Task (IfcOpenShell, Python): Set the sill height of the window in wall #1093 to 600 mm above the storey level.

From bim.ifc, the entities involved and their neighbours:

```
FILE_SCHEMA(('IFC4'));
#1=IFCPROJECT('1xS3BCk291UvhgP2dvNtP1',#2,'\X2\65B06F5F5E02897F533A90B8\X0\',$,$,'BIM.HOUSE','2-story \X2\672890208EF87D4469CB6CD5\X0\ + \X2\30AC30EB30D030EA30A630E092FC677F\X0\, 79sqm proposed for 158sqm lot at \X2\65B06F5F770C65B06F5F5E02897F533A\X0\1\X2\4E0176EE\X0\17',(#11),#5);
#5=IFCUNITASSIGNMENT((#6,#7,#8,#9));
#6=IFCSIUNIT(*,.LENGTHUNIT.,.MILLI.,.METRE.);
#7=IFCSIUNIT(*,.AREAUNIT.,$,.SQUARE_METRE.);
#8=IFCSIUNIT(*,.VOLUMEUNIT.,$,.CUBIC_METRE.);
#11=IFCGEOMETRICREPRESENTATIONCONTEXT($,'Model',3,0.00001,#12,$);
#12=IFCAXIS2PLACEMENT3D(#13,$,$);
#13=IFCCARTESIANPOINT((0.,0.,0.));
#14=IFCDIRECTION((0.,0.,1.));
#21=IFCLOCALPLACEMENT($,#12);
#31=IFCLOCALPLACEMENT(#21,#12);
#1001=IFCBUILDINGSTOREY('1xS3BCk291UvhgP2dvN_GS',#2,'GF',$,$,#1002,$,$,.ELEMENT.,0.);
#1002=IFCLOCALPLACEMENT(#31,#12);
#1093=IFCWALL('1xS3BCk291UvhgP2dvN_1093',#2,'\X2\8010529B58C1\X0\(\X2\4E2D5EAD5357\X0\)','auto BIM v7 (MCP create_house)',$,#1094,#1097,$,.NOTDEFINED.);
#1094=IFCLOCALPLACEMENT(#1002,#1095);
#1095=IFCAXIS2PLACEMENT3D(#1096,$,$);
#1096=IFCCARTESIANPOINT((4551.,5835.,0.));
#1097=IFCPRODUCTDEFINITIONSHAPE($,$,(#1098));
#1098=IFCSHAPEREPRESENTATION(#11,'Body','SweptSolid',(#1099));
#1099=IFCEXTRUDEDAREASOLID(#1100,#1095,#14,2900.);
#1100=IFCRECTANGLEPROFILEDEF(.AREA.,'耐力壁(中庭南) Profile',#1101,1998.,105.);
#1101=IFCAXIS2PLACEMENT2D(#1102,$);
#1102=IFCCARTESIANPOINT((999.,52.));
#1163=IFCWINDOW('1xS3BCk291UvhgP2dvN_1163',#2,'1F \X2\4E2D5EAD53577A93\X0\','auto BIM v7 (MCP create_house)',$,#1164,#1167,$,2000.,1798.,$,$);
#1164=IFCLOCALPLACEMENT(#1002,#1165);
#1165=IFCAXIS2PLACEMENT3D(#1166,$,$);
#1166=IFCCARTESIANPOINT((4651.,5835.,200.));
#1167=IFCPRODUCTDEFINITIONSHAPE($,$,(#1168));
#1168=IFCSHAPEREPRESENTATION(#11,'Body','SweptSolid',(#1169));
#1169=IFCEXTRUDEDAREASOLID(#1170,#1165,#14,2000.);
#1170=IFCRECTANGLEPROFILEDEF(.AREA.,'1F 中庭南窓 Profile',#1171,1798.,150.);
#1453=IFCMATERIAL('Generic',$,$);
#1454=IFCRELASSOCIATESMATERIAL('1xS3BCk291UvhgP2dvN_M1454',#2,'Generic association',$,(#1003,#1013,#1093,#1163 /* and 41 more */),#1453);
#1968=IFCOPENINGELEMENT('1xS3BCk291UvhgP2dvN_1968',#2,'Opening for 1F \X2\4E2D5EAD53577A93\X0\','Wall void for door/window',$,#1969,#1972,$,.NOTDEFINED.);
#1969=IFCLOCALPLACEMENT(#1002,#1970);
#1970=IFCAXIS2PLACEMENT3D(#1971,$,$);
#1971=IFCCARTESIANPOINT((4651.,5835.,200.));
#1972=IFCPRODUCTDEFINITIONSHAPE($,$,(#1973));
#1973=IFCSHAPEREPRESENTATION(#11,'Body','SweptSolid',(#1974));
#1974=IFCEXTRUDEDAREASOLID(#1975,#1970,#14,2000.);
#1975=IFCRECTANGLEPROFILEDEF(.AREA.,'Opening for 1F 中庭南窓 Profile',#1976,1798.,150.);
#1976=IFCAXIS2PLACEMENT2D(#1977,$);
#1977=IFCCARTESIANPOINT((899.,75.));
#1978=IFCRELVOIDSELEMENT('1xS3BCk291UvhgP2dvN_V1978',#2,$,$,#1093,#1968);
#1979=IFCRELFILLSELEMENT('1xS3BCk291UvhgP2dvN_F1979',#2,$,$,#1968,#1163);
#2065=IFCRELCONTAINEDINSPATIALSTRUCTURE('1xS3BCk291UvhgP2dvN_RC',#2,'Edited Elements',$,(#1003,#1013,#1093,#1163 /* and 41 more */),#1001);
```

```python
import numpy as np
import ifcopenshell
import ifcopenshell.api.geometry
import ifcopenshell.geom
import ifcopenshell.util.element
import ifcopenshell.util.placement
import ifcopenshell.util.shape
import ifcopenshell.util.unit

model = ifcopenshell.open("bim.ifc")
unit_scale = ifcopenshell.util.unit.calculate_unit_scale(model)

window = model.by_id(1163)
opening = window.FillsVoids[0].RelatingOpeningElement
storey = ifcopenshell.util.element.get_container(window, ifc_class="IfcBuildingStorey")
level = ifcopenshell.util.placement.get_local_placement(storey.ObjectPlacement)[2, 3]

# The opening's origin need not be at the sill, so measure its lowest point.
shape = ifcopenshell.geom.create_shape(ifcopenshell.geom.settings(), opening)
bottom = ifcopenshell.util.shape.get_shape_bottom_elevation(shape, shape.geometry) / unit_scale
dz = level + 0.6 / unit_scale - bottom

shift = np.array([0.0, 0.0, dz])
# The window is not placed relative to its opening, so move both.
for product in (opening, window):
    matrix = ifcopenshell.util.placement.get_local_placement(product.ObjectPlacement)
    matrix[:3, 3] += shift
    ifcopenshell.api.geometry.edit_object_placement(model, product=product, matrix=matrix, is_si=False)

print(f"moved by {dz * unit_scale:+.3f} m")

model.write("bim_updated.ifc")
```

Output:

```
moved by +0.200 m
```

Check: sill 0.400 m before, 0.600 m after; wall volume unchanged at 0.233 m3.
